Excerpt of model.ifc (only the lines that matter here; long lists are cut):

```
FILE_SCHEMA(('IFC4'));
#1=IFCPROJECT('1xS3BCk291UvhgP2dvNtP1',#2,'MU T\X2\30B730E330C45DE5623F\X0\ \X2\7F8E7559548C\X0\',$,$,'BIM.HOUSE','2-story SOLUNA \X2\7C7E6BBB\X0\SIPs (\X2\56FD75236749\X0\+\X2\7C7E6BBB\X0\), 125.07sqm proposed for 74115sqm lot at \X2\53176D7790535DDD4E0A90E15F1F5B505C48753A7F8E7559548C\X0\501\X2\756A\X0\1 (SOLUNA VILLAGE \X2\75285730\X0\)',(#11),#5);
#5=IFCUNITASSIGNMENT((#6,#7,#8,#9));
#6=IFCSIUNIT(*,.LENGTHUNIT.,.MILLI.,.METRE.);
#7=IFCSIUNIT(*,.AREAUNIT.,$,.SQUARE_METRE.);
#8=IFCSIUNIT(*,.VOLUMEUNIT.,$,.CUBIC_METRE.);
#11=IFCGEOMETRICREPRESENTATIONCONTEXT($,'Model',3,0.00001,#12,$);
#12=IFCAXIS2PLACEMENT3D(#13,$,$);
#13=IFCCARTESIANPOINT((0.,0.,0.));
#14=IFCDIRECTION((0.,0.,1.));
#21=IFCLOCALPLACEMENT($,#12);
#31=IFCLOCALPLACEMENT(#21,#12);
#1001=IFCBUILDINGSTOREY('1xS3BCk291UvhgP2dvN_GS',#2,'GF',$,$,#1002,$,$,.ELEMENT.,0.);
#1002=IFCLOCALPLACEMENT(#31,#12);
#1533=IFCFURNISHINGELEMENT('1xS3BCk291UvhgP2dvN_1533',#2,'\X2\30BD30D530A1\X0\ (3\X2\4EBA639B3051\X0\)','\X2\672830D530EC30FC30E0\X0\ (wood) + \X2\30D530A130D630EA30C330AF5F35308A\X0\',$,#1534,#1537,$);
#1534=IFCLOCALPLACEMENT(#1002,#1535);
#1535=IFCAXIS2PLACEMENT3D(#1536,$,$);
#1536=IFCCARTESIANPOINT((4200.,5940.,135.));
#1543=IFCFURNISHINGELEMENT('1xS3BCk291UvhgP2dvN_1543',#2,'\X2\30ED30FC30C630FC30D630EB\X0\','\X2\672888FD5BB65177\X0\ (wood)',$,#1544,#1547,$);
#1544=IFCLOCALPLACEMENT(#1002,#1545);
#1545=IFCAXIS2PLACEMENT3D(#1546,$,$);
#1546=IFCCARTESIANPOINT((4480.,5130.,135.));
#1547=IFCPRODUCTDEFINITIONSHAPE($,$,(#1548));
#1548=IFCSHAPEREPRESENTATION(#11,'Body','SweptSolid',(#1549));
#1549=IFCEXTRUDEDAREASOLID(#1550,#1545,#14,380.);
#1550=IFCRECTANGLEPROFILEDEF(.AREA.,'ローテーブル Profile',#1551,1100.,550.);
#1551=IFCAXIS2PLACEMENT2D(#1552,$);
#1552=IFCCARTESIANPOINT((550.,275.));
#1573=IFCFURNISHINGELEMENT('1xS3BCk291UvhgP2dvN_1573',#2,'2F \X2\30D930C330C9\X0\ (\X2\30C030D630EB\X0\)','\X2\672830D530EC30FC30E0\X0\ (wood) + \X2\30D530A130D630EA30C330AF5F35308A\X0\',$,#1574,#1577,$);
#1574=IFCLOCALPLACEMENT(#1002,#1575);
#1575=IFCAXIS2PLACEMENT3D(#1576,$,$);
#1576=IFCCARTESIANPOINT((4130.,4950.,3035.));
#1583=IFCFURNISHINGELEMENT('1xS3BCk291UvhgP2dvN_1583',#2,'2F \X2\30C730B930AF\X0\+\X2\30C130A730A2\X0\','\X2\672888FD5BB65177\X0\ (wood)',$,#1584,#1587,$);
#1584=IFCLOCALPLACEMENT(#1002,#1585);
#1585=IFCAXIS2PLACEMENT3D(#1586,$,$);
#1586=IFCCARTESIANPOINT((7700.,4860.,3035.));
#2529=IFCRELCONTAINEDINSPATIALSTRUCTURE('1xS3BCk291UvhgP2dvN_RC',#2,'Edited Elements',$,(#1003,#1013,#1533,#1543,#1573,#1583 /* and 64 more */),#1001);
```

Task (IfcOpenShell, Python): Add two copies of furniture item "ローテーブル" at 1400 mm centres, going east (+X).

```python
import numpy as np
import ifcopenshell
import ifcopenshell.api.geometry
import ifcopenshell.api.root
import ifcopenshell.util.element
import ifcopenshell.util.placement
import ifcopenshell.util.unit

model = ifcopenshell.open("model.ifc")
unit_scale = ifcopenshell.util.unit.calculate_unit_scale(model)


def reuse_history(source, copy):
    """copy_class also copies each property set's owner history, people and application; keep the originals."""
    for rel in copy.IsDefinedBy:
        if rel.is_a("IfcRelDefinesByProperties") and (history := rel.RelatingPropertyDefinition.OwnerHistory):
            rel.RelatingPropertyDefinition.OwnerHistory = source.OwnerHistory
            ifcopenshell.util.element.remove_deep2(model, history)


source = model.by_guid("1xS3BCk291UvhgP2dvN_1543")
base = ifcopenshell.util.placement.get_local_placement(source.ObjectPlacement)
step = np.array([1.0, 0.0, 0.0]) * 1.4 / unit_scale

for i in range(1, 3):
    copy = ifcopenshell.api.root.copy_class(model, product=source)
    copy.Representation = ifcopenshell.util.element.copy_deep(
        model, source.Representation, exclude=["IfcGeometricRepresentationContext", "IfcRepresentationMap"]
    )
    reuse_history(source, copy)
    matrix = base.copy()
    matrix[:3, 3] += i * step
    print("added at", matrix[:3, 3].round(3) + 0.0)
    ifcopenshell.api.geometry.edit_object_placement(model, product=copy, matrix=matrix, is_si=False)

model.write("model_v2.ifc")
```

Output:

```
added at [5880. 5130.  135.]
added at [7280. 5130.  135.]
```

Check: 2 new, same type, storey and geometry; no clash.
